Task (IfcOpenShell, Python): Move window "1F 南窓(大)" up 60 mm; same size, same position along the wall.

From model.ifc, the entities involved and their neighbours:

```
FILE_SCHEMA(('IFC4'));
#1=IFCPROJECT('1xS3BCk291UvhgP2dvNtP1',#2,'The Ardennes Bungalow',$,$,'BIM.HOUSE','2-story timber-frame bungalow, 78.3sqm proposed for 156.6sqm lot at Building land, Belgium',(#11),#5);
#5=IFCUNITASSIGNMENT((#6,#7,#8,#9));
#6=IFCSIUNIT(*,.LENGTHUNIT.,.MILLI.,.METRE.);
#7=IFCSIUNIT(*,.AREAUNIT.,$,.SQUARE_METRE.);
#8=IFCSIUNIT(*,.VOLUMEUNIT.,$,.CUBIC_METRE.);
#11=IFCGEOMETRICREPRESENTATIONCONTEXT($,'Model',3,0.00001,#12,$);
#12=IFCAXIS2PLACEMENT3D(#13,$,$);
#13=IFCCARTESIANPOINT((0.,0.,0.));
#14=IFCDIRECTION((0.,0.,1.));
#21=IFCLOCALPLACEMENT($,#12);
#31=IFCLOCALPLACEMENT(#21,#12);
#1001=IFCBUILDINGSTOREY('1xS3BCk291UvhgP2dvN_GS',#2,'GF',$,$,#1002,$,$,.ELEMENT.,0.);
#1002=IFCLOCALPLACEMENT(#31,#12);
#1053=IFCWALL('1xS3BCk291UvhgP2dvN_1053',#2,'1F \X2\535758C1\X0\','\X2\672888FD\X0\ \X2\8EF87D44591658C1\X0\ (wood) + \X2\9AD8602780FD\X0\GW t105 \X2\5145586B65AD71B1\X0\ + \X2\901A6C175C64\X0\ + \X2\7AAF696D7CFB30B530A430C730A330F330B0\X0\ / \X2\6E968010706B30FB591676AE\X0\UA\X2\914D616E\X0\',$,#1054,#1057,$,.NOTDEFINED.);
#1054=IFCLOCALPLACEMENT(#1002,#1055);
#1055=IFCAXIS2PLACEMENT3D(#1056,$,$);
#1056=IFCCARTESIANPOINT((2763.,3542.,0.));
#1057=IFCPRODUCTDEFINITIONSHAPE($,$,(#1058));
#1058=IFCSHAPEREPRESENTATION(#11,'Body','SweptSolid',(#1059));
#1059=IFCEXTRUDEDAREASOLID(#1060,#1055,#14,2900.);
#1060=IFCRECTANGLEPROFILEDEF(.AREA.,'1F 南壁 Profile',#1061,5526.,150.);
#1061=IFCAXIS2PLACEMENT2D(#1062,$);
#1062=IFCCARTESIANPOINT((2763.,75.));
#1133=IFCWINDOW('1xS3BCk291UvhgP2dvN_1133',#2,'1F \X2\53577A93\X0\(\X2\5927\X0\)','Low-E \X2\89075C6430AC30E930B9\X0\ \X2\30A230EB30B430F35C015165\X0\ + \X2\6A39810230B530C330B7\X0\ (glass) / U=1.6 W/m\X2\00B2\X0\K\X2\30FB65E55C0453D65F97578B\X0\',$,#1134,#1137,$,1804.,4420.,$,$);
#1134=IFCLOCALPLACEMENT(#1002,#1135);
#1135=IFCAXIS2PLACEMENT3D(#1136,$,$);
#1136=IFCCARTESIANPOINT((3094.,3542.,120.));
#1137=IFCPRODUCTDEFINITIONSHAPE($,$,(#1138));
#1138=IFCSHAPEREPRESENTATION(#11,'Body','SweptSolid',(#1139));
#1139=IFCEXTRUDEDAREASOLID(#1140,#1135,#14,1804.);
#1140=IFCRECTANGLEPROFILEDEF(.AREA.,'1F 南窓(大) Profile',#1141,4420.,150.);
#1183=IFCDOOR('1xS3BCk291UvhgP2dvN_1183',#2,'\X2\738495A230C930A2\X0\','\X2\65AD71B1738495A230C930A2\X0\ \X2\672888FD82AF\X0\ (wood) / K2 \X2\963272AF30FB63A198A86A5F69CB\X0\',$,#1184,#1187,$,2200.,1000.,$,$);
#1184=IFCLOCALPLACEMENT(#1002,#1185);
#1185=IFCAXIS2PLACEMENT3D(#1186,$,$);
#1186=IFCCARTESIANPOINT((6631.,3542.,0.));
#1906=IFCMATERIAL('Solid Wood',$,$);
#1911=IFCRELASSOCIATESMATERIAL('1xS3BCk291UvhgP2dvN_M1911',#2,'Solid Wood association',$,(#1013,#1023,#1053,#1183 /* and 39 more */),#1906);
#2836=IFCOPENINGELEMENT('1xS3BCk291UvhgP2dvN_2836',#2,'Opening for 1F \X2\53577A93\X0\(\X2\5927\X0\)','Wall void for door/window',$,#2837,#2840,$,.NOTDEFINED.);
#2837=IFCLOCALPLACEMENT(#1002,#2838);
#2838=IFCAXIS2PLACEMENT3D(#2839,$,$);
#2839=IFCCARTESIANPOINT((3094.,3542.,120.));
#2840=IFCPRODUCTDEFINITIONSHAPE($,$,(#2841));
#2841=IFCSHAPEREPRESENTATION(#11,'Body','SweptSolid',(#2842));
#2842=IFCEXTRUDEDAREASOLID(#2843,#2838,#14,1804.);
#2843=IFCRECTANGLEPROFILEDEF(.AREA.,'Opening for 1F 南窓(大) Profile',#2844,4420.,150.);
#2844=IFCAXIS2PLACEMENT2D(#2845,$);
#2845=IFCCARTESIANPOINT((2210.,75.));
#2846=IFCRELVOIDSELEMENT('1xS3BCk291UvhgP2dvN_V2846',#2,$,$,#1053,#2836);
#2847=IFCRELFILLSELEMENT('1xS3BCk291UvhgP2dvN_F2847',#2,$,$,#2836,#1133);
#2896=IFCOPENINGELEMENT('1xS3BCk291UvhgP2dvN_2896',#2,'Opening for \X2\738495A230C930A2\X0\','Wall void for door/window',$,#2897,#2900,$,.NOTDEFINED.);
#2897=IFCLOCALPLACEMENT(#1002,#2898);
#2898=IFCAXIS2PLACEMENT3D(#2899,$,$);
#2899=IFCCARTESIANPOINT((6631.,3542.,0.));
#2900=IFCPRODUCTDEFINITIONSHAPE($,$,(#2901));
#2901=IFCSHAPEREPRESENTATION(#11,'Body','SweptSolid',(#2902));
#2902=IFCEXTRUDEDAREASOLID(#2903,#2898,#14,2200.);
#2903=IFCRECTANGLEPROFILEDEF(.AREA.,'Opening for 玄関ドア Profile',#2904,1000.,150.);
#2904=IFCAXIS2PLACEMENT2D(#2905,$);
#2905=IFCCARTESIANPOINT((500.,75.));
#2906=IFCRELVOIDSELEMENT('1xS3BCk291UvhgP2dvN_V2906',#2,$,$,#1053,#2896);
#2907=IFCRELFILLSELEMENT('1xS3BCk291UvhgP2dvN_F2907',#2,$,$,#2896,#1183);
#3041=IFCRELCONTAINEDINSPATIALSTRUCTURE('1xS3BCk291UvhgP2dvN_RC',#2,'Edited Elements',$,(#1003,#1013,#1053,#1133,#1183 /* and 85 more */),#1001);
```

```python
import numpy as np
import ifcopenshell
import ifcopenshell.api.geometry
import ifcopenshell.util.placement
import ifcopenshell.util.unit

model = ifcopenshell.open("model.ifc")
unit_scale = ifcopenshell.util.unit.calculate_unit_scale(model)

window = model.by_guid("1xS3BCk291UvhgP2dvN_1133")
opening = window.FillsVoids[0].RelatingOpeningElement
dz = 0.06 / unit_scale

shift = np.array([0.0, 0.0, dz])
# The window is not placed relative to its opening, so move both.
for product in (opening, window):
    matrix = ifcopenshell.util.placement.get_local_placement(product.ObjectPlacement)
    matrix[:3, 3] += shift
    ifcopenshell.api.geometry.edit_object_placement(model, product=product, matrix=matrix, is_si=False)

print(f"moved by {dz * unit_scale:+.3f} m")

model.write("model_v2.ifc")
```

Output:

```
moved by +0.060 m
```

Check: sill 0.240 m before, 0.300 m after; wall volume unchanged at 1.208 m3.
